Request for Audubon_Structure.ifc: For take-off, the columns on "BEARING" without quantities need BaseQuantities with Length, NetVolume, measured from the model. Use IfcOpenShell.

First a look at what the model holds.

```python
import ifcopenshell
import ifcopenshell.util.element
import ifcopenshell.util.unit

model = ifcopenshell.open("Audubon_Structure.ifc")
print(model.schema)
for unit_type in ("LENGTHUNIT", "AREAUNIT", "VOLUMEUNIT"):
    print(unit_type, ifcopenshell.util.unit.calculate_unit_scale(model, unit_type))
storey = next(s for s in model.by_type("IfcBuildingStorey") if s.Name == "BEARING")
columns = [e for e in ifcopenshell.util.element.get_decomposition(storey) if e.is_a("IfcColumn")]
for e in sorted(columns, key=lambda e: e.id()):
    print(e.id(), e.is_a(), e.Name, list(ifcopenshell.util.element.get_psets(e, qtos_only=True)), sep=" | ")
```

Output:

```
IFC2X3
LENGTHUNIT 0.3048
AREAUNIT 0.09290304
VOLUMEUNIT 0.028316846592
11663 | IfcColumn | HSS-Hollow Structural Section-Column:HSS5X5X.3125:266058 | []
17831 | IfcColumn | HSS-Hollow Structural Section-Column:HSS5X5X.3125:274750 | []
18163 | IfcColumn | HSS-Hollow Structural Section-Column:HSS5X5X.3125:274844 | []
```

```python
import ifcopenshell
import ifcopenshell.api.pset
import ifcopenshell.geom
import ifcopenshell.util.element
import ifcopenshell.util.shape
import ifcopenshell.util.unit

model = ifcopenshell.open("Audubon_Structure.ifc")
unit_scale = ifcopenshell.util.unit.calculate_unit_scale(model)
volume_scale = ifcopenshell.util.unit.calculate_unit_scale(model, "VOLUMEUNIT")
settings = ifcopenshell.geom.settings()

storey = next(s for s in model.by_type("IfcBuildingStorey") if s.Name == "BEARING")
columns = [e for e in ifcopenshell.util.element.get_decomposition(storey) if e.is_a("IfcColumn")]

for e in sorted(columns, key=lambda e: e.id()):
    if ifcopenshell.util.element.get_psets(e, qtos_only=True, should_inherit=False):
        continue
    # Geometry comes back in metres, in the element's own axes.
    shape = ifcopenshell.geom.create_shape(settings, e)
    values = {
        "Length": ifcopenshell.util.shape.get_z(shape.geometry) / unit_scale,
        "NetVolume": ifcopenshell.util.shape.get_volume(shape.geometry) / volume_scale,
    }
    qto = ifcopenshell.api.pset.add_qto(model, product=e, name="BaseQuantities")
    ifcopenshell.api.pset.edit_qto(model, qto=qto, properties=values)
    print(e.id(), {k: round(v, 3) for k, v in values.items()})

model.write("Audubon_Structure_rev.ifc")
```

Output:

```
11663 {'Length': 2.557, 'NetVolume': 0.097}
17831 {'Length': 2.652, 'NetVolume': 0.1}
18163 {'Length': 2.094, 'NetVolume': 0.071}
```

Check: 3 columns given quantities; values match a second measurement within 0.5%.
